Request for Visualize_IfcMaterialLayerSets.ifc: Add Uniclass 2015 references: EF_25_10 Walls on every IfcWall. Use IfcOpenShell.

First a look at what the model holds.

```python
import ifcopenshell

model = ifcopenshell.open("Visualize_IfcMaterialLayerSets.ifc")
print(model.schema)
print("classifications:", [c.Name for c in model.by_type("IfcClassification")])
for ifc_class in ("IfcDoor", "IfcRoof", "IfcStair", "IfcWall", "IfcWindow"):
    print(ifc_class, len(model.by_type(ifc_class)))
```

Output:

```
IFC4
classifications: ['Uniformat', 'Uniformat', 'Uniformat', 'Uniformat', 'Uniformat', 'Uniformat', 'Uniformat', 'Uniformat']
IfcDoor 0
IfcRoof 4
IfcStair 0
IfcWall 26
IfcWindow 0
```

```python
import ifcopenshell
import ifcopenshell.api.classification

model = ifcopenshell.open("Visualize_IfcMaterialLayerSets.ifc")

system = ifcopenshell.api.classification.add_classification(model, classification="Uniclass 2015")

codes = {
    "IfcWall": ("EF_25_10", "Walls"),
}
for ifc_class, (code, name) in codes.items():
    products = model.by_type(ifc_class)
    ifcopenshell.api.classification.add_reference(
        model, products=products, classification=system, identification=code, name=name
    )
    print(code, len(products))

model.write("Visualize_IfcMaterialLayerSets_edited.ifc")
```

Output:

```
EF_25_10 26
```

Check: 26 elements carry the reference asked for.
